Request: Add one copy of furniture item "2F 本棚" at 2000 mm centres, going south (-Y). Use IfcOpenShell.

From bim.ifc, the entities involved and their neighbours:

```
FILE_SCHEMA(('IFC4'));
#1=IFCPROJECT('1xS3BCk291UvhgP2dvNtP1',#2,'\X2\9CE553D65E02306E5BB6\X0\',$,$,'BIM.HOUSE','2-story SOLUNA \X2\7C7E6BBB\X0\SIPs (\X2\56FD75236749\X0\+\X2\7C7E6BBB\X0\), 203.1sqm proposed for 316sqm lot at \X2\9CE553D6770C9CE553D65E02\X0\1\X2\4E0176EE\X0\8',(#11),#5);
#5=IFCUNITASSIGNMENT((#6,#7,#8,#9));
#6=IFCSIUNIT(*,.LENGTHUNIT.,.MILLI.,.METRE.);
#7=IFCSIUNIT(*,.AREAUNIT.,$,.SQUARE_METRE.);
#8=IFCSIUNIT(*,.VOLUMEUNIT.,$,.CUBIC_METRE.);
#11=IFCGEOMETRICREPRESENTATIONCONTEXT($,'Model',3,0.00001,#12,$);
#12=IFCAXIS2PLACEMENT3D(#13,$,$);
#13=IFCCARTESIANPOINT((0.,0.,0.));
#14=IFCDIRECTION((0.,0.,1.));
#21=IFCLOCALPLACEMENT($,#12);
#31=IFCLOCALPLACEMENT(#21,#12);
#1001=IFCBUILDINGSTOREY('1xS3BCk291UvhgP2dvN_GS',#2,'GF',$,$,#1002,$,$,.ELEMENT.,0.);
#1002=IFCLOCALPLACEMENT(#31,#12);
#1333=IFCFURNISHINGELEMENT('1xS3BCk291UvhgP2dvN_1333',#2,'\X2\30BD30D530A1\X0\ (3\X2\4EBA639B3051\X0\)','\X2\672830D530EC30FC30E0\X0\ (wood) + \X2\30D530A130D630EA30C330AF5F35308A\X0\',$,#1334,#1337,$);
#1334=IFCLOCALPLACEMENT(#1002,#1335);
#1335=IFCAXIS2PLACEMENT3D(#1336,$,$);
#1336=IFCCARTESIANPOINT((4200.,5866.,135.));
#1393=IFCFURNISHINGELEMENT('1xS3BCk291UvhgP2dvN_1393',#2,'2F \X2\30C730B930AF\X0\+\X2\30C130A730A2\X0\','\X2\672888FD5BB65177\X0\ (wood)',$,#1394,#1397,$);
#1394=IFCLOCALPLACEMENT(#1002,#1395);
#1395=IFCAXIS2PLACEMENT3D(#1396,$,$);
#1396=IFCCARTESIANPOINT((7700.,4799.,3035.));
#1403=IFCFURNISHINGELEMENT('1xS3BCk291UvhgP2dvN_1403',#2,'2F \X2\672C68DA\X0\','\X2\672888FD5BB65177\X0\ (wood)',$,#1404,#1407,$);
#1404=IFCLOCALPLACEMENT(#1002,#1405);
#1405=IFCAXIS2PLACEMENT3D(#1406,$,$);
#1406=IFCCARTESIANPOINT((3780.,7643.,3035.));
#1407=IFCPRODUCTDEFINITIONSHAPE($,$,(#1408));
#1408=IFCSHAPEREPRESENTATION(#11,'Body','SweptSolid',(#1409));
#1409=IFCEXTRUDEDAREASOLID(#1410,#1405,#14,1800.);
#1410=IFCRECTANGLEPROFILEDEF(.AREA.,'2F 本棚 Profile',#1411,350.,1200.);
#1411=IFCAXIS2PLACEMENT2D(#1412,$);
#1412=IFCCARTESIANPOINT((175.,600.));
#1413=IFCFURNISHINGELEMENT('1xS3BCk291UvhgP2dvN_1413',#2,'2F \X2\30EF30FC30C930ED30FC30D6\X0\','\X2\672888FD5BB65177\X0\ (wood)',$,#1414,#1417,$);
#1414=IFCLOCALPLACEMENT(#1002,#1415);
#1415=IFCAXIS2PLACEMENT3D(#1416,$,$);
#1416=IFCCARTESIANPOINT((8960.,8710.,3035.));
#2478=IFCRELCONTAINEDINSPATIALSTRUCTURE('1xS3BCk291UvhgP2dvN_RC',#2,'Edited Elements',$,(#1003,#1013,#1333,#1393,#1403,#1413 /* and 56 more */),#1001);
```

```python
import numpy as np
import ifcopenshell
import ifcopenshell.api.geometry
import ifcopenshell.api.root
import ifcopenshell.util.element
import ifcopenshell.util.placement

model = ifcopenshell.open("bim.ifc")


def reuse_history(source, copy):
    """copy_class also copies each property set's owner history, people and application; keep the originals."""
    for rel in copy.IsDefinedBy:
        if rel.is_a("IfcRelDefinesByProperties") and (history := rel.RelatingPropertyDefinition.OwnerHistory):
            rel.RelatingPropertyDefinition.OwnerHistory = source.OwnerHistory
            ifcopenshell.util.element.remove_deep2(model, history)


source = model.by_guid("1xS3BCk291UvhgP2dvN_1403")
base = ifcopenshell.util.placement.get_local_placement(source.ObjectPlacement)
step = np.array([0.0, -1.0, 0.0]) * 2000.0

for i in range(1, 2):
    copy = ifcopenshell.api.root.copy_class(model, product=source)
    copy.Representation = ifcopenshell.util.element.copy_deep(
        model, source.Representation, exclude=["IfcGeometricRepresentationContext", "IfcRepresentationMap"]
    )
    reuse_history(source, copy)
    matrix = base.copy()
    matrix[:3, 3] += i * step
    print("added at", matrix[:3, 3].round(3) + 0.0)
    ifcopenshell.api.geometry.edit_object_placement(model, product=copy, matrix=matrix, is_si=False)

model.write("bim_rev.ifc")
```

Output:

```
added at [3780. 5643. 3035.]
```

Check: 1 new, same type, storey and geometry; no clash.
